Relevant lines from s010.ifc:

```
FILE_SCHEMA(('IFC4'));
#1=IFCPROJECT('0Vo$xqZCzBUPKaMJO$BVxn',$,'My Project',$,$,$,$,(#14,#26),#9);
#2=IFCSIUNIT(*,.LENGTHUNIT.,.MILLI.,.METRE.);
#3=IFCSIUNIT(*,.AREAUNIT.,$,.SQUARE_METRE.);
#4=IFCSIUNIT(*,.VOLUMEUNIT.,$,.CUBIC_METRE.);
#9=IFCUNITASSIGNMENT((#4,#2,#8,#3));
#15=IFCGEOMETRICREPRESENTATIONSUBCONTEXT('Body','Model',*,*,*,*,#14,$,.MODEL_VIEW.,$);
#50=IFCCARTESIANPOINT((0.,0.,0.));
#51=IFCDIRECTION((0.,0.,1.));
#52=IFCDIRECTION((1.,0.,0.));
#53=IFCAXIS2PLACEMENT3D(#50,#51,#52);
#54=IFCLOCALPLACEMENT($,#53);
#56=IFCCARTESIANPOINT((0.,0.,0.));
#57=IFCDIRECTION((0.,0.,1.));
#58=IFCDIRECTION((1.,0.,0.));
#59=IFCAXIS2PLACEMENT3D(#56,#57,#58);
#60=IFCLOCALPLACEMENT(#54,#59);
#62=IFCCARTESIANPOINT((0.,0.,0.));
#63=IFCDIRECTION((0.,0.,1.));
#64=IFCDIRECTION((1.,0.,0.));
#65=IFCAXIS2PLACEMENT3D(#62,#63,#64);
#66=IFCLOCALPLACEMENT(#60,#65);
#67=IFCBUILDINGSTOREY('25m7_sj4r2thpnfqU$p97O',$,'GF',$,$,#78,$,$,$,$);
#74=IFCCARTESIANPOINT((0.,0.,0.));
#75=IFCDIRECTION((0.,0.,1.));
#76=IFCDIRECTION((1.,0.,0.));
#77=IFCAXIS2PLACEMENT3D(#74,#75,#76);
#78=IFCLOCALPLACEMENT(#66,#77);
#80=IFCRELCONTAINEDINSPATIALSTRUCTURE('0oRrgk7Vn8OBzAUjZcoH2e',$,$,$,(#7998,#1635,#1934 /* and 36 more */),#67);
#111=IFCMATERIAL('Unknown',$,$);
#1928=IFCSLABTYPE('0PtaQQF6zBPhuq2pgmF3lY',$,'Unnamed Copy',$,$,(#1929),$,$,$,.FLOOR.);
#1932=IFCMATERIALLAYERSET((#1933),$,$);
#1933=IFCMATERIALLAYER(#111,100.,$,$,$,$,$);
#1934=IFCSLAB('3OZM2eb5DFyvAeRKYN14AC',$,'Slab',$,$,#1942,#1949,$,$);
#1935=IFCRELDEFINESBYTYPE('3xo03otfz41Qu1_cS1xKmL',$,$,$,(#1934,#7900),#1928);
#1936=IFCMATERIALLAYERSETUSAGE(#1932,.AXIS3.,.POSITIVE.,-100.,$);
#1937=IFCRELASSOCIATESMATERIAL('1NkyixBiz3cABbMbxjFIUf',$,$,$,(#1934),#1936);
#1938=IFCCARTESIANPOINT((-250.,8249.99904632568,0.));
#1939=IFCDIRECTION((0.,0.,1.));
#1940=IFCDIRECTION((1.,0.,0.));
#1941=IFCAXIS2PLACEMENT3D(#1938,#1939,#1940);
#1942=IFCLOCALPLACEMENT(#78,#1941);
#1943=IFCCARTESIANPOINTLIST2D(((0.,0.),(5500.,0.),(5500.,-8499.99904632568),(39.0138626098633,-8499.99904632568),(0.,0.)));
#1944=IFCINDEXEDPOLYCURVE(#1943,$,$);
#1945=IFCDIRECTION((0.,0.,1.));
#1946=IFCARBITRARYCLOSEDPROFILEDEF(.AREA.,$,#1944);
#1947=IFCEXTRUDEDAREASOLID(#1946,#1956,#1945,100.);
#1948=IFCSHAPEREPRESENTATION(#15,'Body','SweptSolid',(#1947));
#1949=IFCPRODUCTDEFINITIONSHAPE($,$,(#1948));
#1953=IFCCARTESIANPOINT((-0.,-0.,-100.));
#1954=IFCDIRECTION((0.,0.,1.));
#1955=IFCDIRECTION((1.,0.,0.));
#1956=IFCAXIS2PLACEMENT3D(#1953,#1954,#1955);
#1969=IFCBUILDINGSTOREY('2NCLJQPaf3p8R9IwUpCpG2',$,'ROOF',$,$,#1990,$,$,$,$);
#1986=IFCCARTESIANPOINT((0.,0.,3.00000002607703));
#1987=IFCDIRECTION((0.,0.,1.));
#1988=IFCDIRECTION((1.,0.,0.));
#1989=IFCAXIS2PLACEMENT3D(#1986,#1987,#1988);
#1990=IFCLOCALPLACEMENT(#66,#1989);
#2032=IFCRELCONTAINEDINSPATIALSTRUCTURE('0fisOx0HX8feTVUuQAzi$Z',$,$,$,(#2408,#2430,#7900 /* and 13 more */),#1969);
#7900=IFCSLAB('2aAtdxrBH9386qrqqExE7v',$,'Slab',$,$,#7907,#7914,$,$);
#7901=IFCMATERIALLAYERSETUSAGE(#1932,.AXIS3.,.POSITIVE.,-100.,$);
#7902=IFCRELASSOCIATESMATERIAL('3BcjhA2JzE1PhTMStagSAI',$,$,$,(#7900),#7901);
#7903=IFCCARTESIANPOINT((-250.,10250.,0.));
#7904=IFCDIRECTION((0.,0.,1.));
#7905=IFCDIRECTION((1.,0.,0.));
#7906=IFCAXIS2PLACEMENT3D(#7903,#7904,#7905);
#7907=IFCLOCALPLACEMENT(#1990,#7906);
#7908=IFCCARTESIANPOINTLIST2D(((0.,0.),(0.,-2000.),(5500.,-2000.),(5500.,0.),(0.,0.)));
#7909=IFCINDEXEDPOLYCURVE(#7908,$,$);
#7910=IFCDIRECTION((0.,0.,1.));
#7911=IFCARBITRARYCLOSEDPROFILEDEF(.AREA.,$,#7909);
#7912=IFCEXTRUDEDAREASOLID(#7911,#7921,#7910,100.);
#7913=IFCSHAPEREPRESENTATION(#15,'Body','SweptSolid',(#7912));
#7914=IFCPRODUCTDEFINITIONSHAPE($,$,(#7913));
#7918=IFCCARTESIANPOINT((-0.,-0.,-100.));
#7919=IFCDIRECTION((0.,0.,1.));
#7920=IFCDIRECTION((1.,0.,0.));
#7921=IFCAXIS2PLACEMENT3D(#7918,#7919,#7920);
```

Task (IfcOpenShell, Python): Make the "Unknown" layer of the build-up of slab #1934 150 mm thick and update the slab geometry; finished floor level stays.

```python
import ifcopenshell
import ifcopenshell.util.element
import ifcopenshell.util.representation
import ifcopenshell.util.unit

model = ifcopenshell.open("s010.ifc")
unit_scale = ifcopenshell.util.unit.calculate_unit_scale(model)

layer_set = model.by_id(1932)
layer = next(l for l in layer_set.MaterialLayers if l.Material and l.Material.Name == "Unknown")
change = 0.15 / unit_scale - layer.LayerThickness
layer.LayerThickness += change

# The layer set is shared, so every slab that uses it gets the new thickness.
slabs = [e for e in ifcopenshell.util.element.get_elements_by_material(model, layer_set) if e.is_a("IfcSlab")]
for slab in sorted(slabs, key=lambda e: e.id()):
    body = ifcopenshell.util.representation.get_representation(slab, "Model", "Body")
    solid = body.Items[0]
    old_depth = solid.Depth
    solid.Depth += change
    # Extruded upwards: lower the start of the extrusion so the top stays.
    x, y, z = solid.Position.Location.Coordinates
    solid.Position.Location = model.createIfcCartesianPoint((x, y, z - change))
    print(slab.id(), f"{old_depth:g} -> {solid.Depth:g}")

# The layers are counted up from the underside, which has moved.
for usage in {ifcopenshell.util.element.get_material(slab) for slab in slabs}:
    usage.OffsetFromReferenceLine -= change

model.write("s010_v2.ifc")
```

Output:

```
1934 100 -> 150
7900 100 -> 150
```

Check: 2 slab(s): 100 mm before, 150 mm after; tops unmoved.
